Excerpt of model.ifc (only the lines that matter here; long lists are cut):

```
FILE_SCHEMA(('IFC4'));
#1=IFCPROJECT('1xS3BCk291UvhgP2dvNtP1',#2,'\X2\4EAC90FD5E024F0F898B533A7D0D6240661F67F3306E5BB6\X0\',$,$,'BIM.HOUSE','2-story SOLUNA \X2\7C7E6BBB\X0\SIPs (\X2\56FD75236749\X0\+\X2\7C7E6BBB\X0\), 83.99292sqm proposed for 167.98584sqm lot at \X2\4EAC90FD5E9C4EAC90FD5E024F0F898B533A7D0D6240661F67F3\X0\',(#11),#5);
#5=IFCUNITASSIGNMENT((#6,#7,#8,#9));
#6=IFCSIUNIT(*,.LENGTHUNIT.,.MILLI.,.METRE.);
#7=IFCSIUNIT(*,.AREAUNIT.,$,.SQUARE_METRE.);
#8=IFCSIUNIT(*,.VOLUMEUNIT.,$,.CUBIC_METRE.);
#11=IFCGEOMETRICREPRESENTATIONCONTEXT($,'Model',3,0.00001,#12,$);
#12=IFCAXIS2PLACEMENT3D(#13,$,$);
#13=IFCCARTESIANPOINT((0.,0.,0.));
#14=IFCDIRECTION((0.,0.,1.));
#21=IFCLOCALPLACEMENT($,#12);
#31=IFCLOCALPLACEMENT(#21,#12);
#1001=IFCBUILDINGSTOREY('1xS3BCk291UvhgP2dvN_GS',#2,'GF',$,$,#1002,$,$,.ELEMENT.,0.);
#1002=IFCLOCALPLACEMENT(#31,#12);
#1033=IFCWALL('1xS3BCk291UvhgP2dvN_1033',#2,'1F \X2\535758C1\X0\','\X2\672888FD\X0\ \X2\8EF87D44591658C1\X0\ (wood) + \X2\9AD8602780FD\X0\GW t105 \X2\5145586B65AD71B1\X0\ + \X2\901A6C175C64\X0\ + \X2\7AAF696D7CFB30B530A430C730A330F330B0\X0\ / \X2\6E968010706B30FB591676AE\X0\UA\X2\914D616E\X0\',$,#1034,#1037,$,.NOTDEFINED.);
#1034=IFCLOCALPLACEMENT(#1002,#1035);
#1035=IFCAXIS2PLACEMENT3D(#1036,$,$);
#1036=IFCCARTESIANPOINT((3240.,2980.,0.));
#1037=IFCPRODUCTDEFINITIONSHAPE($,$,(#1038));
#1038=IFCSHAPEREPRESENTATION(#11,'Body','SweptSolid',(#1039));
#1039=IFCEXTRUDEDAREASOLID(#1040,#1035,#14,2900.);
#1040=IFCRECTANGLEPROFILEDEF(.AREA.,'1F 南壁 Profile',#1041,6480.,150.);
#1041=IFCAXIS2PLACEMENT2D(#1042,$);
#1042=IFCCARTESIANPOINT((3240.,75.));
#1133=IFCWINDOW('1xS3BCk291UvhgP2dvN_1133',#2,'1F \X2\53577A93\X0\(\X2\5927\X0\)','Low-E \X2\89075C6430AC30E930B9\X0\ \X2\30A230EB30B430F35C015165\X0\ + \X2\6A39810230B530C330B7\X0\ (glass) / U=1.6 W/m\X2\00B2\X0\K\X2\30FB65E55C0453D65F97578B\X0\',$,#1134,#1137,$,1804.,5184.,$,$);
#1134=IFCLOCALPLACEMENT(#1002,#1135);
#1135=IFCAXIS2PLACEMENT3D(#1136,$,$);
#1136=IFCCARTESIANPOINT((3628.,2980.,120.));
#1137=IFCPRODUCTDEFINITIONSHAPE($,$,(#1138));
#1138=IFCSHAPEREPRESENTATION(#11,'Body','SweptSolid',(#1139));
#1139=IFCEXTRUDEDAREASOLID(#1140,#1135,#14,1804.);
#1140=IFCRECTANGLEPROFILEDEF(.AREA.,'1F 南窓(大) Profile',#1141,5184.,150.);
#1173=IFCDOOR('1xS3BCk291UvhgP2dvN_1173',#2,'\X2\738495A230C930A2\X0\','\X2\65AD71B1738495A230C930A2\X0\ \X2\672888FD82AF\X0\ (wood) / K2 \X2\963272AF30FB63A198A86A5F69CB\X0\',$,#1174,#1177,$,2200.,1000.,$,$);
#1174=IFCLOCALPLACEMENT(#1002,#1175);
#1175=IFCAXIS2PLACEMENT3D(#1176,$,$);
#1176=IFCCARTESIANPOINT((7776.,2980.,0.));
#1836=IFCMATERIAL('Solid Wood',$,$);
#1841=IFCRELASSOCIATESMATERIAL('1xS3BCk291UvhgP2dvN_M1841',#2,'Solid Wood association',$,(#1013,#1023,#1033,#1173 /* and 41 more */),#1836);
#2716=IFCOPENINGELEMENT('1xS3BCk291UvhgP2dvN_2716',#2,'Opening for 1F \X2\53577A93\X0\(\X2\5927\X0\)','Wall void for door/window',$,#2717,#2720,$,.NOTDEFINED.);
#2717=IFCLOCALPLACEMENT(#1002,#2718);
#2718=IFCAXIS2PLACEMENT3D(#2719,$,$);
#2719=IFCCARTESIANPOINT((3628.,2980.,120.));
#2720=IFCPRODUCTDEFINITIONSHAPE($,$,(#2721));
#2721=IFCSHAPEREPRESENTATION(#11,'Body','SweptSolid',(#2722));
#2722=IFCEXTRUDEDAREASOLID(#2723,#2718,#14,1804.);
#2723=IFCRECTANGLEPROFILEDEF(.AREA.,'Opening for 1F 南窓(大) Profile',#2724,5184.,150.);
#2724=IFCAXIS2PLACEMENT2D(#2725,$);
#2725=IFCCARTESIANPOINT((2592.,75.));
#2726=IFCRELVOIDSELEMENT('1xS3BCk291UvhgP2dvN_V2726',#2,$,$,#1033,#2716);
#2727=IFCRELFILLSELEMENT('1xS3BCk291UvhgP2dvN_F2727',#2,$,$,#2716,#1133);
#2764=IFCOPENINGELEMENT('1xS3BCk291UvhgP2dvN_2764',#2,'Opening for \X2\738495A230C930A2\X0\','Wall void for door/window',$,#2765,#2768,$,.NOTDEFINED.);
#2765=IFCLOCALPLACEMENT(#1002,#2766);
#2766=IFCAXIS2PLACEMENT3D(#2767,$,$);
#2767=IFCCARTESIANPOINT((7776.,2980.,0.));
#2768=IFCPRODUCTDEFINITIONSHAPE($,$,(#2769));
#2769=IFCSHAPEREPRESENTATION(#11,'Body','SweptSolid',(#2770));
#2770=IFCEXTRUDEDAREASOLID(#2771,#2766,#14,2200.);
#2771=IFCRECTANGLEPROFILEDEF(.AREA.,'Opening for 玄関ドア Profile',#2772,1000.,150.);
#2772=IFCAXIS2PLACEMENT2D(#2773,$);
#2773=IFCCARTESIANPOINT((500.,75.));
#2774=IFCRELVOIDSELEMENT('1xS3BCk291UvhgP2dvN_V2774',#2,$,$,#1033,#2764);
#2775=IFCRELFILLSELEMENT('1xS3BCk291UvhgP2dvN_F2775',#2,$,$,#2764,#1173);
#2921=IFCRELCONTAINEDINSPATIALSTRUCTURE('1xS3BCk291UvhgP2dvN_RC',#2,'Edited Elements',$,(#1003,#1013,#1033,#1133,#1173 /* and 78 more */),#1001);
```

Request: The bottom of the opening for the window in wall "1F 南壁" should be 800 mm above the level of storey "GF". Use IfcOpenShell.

```python
import numpy as np
import ifcopenshell
import ifcopenshell.api.geometry
import ifcopenshell.geom
import ifcopenshell.util.element
import ifcopenshell.util.placement
import ifcopenshell.util.shape
import ifcopenshell.util.unit

model = ifcopenshell.open("model.ifc")
unit_scale = ifcopenshell.util.unit.calculate_unit_scale(model)

window = model.by_id(1133)
opening = window.FillsVoids[0].RelatingOpeningElement
storey = ifcopenshell.util.element.get_container(window, ifc_class="IfcBuildingStorey")
level = ifcopenshell.util.placement.get_local_placement(storey.ObjectPlacement)[2, 3]

# The opening's origin need not be at the sill, so measure its lowest point.
shape = ifcopenshell.geom.create_shape(ifcopenshell.geom.settings(), opening)
bottom = ifcopenshell.util.shape.get_shape_bottom_elevation(shape, shape.geometry) / unit_scale
dz = level + 0.8 / unit_scale - bottom

shift = np.array([0.0, 0.0, dz])
# The window is not placed relative to its opening, so move both.
for product in (opening, window):
    matrix = ifcopenshell.util.placement.get_local_placement(product.ObjectPlacement)
    matrix[:3, 3] += shift
    ifcopenshell.api.geometry.edit_object_placement(model, product=product, matrix=matrix, is_si=False)

print(f"moved by {dz * unit_scale:+.3f} m")

model.write("model_updated.ifc")
```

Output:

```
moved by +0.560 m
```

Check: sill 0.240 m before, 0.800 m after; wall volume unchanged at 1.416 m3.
